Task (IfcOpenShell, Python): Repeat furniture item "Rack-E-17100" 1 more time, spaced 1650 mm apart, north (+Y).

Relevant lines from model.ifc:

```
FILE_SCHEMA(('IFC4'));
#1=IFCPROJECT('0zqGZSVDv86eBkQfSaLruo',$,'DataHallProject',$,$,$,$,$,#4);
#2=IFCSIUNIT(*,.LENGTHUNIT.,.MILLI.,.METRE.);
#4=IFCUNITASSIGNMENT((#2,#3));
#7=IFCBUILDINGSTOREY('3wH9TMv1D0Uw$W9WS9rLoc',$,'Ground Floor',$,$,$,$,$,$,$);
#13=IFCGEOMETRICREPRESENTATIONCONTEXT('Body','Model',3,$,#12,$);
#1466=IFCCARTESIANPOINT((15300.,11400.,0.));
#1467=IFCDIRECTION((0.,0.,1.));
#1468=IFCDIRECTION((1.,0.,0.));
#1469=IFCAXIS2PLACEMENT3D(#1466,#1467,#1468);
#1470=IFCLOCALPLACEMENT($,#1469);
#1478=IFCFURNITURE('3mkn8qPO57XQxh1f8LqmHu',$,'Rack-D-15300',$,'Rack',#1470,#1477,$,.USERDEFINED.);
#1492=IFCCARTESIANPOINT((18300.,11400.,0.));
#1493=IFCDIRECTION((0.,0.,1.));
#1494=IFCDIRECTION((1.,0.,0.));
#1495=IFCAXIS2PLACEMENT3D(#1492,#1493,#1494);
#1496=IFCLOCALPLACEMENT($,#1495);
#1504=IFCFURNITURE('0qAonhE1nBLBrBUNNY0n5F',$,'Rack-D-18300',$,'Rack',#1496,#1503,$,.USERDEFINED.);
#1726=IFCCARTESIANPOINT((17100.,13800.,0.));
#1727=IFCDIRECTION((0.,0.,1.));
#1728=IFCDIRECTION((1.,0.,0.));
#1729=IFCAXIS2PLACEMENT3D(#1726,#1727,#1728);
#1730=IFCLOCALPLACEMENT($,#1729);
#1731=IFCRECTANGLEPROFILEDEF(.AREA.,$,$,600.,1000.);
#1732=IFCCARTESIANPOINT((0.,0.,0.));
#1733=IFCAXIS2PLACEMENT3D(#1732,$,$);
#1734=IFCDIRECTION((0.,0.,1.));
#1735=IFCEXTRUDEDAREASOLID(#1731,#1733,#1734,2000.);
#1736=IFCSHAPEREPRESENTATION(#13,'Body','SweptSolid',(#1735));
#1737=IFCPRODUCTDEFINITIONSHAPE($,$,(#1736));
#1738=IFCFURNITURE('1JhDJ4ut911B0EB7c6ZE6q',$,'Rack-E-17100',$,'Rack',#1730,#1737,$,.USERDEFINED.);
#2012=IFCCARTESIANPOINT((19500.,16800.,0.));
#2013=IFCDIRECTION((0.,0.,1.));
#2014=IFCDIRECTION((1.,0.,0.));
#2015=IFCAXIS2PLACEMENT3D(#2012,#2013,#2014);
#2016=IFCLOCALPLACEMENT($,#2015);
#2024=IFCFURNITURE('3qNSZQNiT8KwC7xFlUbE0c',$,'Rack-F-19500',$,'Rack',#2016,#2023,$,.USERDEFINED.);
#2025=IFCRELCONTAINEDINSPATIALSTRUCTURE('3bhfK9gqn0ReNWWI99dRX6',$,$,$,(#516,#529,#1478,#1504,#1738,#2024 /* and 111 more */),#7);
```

```python
import numpy as np
import ifcopenshell
import ifcopenshell.api.geometry
import ifcopenshell.api.root
import ifcopenshell.util.element
import ifcopenshell.util.placement
import ifcopenshell.util.unit

model = ifcopenshell.open("model.ifc")
unit_scale = ifcopenshell.util.unit.calculate_unit_scale(model)

source = model.by_guid("1JhDJ4ut911B0EB7c6ZE6q")
base = ifcopenshell.util.placement.get_local_placement(source.ObjectPlacement)
step = np.array([0.0, 1.0, 0.0]) * 1.65 / unit_scale

for i in range(1, 2):
    copy = ifcopenshell.api.root.copy_class(model, product=source)
    copy.Representation = ifcopenshell.util.element.copy_deep(
        model, source.Representation, exclude=["IfcGeometricRepresentationContext", "IfcRepresentationMap"]
    )
    matrix = base.copy()
    matrix[:3, 3] += i * step
    print("added at", matrix[:3, 3].round(3) + 0.0)
    ifcopenshell.api.geometry.edit_object_placement(model, product=copy, matrix=matrix, is_si=False)

model.write("model_updated.ifc")
```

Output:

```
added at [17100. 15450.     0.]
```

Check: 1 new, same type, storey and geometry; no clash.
